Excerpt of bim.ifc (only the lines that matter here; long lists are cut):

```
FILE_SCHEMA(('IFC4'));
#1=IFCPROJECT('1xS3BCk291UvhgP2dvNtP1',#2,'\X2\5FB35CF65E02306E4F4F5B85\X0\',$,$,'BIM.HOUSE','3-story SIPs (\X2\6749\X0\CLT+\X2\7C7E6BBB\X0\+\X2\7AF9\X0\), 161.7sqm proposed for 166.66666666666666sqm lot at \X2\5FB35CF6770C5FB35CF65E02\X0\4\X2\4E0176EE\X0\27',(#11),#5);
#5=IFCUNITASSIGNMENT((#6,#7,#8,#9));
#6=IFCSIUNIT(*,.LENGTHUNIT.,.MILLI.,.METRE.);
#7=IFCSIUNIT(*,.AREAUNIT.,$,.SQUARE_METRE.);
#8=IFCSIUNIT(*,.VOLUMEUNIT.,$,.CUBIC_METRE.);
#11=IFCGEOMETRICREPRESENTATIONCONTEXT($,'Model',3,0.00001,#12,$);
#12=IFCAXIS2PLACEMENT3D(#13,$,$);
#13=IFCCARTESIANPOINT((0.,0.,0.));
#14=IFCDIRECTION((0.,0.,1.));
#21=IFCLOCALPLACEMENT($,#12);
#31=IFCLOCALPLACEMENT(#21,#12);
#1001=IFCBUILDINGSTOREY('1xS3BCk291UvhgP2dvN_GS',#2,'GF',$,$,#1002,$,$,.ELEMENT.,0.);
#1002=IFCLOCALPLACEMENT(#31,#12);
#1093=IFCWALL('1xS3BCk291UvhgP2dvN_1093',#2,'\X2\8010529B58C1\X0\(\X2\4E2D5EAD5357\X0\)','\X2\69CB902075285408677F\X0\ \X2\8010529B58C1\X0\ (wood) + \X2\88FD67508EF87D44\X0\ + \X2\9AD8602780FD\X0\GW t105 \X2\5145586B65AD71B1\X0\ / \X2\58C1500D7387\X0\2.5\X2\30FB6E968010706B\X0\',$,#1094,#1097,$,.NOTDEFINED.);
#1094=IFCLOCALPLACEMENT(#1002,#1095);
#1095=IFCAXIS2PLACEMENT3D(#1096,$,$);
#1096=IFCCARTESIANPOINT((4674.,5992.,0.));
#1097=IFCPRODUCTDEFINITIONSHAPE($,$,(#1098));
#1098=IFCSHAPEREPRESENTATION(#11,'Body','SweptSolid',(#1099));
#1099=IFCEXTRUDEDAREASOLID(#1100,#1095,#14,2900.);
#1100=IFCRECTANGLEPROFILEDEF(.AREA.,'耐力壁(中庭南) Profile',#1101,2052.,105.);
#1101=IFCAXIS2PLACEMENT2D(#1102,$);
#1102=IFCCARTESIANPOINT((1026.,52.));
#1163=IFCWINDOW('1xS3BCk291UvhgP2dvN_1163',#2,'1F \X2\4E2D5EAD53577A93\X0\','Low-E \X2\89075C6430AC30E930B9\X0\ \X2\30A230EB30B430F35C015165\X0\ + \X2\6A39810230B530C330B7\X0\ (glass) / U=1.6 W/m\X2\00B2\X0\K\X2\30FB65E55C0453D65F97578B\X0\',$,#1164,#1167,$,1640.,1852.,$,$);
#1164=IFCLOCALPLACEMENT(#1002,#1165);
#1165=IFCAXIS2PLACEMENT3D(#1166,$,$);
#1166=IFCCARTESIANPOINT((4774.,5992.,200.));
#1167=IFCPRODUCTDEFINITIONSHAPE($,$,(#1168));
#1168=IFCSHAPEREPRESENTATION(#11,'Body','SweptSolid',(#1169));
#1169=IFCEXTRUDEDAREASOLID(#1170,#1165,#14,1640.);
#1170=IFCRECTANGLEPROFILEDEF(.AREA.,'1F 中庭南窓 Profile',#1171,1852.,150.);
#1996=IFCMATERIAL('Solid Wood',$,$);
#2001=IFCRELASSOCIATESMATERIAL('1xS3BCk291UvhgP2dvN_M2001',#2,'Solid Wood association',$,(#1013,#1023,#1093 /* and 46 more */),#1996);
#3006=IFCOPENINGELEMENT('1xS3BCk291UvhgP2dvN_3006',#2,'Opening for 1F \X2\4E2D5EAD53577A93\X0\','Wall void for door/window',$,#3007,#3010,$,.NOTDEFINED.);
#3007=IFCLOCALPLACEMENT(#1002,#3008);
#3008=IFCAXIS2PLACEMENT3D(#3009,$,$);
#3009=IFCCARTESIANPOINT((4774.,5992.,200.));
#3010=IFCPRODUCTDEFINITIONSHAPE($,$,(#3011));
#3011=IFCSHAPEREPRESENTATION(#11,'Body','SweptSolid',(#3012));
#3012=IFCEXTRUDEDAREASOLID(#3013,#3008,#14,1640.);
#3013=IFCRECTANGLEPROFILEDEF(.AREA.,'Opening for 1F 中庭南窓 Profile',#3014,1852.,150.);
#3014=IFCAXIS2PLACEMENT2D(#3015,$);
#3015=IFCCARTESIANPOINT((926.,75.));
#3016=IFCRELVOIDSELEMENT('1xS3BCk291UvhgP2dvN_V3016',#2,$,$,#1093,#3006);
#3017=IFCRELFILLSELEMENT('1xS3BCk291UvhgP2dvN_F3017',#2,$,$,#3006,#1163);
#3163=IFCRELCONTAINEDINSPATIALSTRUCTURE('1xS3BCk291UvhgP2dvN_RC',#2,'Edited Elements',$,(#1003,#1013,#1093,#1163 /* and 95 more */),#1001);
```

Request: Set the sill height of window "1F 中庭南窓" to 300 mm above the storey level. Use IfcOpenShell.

```python
import numpy as np
import ifcopenshell
import ifcopenshell.api.geometry
import ifcopenshell.geom
import ifcopenshell.util.element
import ifcopenshell.util.placement
import ifcopenshell.util.shape
import ifcopenshell.util.unit

model = ifcopenshell.open("bim.ifc")
unit_scale = ifcopenshell.util.unit.calculate_unit_scale(model)

window = model.by_id(1163)
opening = window.FillsVoids[0].RelatingOpeningElement
storey = ifcopenshell.util.element.get_container(window, ifc_class="IfcBuildingStorey")
level = ifcopenshell.util.placement.get_local_placement(storey.ObjectPlacement)[2, 3]

# The opening's origin need not be at the sill, so measure its lowest point.
shape = ifcopenshell.geom.create_shape(ifcopenshell.geom.settings(), opening)
bottom = ifcopenshell.util.shape.get_shape_bottom_elevation(shape, shape.geometry) / unit_scale
dz = level + 0.3 / unit_scale - bottom

shift = np.array([0.0, 0.0, dz])
# The window is not placed relative to its opening, so move both.
for product in (opening, window):
    matrix = ifcopenshell.util.placement.get_local_placement(product.ObjectPlacement)
    matrix[:3, 3] += shift
    ifcopenshell.api.geometry.edit_object_placement(model, product=product, matrix=matrix, is_si=False)

print(f"moved by {dz * unit_scale:+.3f} m")

model.write("bim-out.ifc")
```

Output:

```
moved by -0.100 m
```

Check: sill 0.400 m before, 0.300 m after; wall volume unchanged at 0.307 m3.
